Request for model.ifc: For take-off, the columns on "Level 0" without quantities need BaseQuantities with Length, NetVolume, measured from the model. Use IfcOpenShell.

First a look at what the model holds.

```python
import ifcopenshell
import ifcopenshell.util.element
import ifcopenshell.util.unit

model = ifcopenshell.open("model.ifc")
print(model.schema)
for unit_type in ("LENGTHUNIT", "AREAUNIT", "VOLUMEUNIT"):
    print(unit_type, ifcopenshell.util.unit.calculate_unit_scale(model, unit_type))
storey = next(s for s in model.by_type("IfcBuildingStorey") if s.Name == "Level 0")
columns = [e for e in ifcopenshell.util.element.get_decomposition(storey) if e.is_a("IfcColumn")]
for e in sorted(columns, key=lambda e: e.id()):
    print(e.id(), e.is_a(), e.Name, list(ifcopenshell.util.element.get_psets(e, qtos_only=True)), sep=" | ")
```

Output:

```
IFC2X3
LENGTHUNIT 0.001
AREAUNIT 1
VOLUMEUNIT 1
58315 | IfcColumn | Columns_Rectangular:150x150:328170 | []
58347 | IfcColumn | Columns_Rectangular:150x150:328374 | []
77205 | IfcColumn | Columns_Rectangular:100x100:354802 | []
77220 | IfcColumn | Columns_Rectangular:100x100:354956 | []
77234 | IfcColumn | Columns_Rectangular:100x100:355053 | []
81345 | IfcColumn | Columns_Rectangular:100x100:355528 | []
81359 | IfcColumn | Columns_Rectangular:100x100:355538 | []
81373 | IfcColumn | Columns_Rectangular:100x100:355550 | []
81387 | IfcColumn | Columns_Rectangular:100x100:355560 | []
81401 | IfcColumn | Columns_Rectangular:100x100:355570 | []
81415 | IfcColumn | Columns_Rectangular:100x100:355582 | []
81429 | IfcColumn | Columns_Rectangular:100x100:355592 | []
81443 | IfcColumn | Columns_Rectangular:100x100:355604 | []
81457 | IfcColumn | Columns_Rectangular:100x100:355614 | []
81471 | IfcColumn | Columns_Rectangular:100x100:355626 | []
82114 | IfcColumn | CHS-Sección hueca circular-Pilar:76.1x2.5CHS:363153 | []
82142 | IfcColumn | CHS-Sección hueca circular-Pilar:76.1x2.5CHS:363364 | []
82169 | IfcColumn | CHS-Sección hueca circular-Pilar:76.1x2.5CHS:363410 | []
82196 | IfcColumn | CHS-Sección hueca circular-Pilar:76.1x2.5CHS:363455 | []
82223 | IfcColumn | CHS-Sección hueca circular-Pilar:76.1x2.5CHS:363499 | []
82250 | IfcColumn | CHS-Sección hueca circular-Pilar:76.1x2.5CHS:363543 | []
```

```python
import ifcopenshell
import ifcopenshell.api.pset
import ifcopenshell.geom
import ifcopenshell.util.element
import ifcopenshell.util.shape
import ifcopenshell.util.unit

model = ifcopenshell.open("model.ifc")
unit_scale = ifcopenshell.util.unit.calculate_unit_scale(model)
volume_scale = ifcopenshell.util.unit.calculate_unit_scale(model, "VOLUMEUNIT")
settings = ifcopenshell.geom.settings()

storey = next(s for s in model.by_type("IfcBuildingStorey") if s.Name == "Level 0")
columns = [e for e in ifcopenshell.util.element.get_decomposition(storey) if e.is_a("IfcColumn")]

for e in sorted(columns, key=lambda e: e.id()):
    if ifcopenshell.util.element.get_psets(e, qtos_only=True, should_inherit=False):
        continue
    # Geometry comes back in metres, in the element's own axes.
    shape = ifcopenshell.geom.create_shape(settings, e)
    values = {
        "Length": ifcopenshell.util.shape.get_z(shape.geometry) / unit_scale,
        "NetVolume": ifcopenshell.util.shape.get_volume(shape.geometry) / volume_scale,
    }
    qto = ifcopenshell.api.pset.add_qto(model, product=e, name="BaseQuantities")
    ifcopenshell.api.pset.edit_qto(model, qto=qto, properties=values)
    print(e.id(), {k: round(v, 3) for k, v in values.items()})

model.write("model_v2.ifc")
```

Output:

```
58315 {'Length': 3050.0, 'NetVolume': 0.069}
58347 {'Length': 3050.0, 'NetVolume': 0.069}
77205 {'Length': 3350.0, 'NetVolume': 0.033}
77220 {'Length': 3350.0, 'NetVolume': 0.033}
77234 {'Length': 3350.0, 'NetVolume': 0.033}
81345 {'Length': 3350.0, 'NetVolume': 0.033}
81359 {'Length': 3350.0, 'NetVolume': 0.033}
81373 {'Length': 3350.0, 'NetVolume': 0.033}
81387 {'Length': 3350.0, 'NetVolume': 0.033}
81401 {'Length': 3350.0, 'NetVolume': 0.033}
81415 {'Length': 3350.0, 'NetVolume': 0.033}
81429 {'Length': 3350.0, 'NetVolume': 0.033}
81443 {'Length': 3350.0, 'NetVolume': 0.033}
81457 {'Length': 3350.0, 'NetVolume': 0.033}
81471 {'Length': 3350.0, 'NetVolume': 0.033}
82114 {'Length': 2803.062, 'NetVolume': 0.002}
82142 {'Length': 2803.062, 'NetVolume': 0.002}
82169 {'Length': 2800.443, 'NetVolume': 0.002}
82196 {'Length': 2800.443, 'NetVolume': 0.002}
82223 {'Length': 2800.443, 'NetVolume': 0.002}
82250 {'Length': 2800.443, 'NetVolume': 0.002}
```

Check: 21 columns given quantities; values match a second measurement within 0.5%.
